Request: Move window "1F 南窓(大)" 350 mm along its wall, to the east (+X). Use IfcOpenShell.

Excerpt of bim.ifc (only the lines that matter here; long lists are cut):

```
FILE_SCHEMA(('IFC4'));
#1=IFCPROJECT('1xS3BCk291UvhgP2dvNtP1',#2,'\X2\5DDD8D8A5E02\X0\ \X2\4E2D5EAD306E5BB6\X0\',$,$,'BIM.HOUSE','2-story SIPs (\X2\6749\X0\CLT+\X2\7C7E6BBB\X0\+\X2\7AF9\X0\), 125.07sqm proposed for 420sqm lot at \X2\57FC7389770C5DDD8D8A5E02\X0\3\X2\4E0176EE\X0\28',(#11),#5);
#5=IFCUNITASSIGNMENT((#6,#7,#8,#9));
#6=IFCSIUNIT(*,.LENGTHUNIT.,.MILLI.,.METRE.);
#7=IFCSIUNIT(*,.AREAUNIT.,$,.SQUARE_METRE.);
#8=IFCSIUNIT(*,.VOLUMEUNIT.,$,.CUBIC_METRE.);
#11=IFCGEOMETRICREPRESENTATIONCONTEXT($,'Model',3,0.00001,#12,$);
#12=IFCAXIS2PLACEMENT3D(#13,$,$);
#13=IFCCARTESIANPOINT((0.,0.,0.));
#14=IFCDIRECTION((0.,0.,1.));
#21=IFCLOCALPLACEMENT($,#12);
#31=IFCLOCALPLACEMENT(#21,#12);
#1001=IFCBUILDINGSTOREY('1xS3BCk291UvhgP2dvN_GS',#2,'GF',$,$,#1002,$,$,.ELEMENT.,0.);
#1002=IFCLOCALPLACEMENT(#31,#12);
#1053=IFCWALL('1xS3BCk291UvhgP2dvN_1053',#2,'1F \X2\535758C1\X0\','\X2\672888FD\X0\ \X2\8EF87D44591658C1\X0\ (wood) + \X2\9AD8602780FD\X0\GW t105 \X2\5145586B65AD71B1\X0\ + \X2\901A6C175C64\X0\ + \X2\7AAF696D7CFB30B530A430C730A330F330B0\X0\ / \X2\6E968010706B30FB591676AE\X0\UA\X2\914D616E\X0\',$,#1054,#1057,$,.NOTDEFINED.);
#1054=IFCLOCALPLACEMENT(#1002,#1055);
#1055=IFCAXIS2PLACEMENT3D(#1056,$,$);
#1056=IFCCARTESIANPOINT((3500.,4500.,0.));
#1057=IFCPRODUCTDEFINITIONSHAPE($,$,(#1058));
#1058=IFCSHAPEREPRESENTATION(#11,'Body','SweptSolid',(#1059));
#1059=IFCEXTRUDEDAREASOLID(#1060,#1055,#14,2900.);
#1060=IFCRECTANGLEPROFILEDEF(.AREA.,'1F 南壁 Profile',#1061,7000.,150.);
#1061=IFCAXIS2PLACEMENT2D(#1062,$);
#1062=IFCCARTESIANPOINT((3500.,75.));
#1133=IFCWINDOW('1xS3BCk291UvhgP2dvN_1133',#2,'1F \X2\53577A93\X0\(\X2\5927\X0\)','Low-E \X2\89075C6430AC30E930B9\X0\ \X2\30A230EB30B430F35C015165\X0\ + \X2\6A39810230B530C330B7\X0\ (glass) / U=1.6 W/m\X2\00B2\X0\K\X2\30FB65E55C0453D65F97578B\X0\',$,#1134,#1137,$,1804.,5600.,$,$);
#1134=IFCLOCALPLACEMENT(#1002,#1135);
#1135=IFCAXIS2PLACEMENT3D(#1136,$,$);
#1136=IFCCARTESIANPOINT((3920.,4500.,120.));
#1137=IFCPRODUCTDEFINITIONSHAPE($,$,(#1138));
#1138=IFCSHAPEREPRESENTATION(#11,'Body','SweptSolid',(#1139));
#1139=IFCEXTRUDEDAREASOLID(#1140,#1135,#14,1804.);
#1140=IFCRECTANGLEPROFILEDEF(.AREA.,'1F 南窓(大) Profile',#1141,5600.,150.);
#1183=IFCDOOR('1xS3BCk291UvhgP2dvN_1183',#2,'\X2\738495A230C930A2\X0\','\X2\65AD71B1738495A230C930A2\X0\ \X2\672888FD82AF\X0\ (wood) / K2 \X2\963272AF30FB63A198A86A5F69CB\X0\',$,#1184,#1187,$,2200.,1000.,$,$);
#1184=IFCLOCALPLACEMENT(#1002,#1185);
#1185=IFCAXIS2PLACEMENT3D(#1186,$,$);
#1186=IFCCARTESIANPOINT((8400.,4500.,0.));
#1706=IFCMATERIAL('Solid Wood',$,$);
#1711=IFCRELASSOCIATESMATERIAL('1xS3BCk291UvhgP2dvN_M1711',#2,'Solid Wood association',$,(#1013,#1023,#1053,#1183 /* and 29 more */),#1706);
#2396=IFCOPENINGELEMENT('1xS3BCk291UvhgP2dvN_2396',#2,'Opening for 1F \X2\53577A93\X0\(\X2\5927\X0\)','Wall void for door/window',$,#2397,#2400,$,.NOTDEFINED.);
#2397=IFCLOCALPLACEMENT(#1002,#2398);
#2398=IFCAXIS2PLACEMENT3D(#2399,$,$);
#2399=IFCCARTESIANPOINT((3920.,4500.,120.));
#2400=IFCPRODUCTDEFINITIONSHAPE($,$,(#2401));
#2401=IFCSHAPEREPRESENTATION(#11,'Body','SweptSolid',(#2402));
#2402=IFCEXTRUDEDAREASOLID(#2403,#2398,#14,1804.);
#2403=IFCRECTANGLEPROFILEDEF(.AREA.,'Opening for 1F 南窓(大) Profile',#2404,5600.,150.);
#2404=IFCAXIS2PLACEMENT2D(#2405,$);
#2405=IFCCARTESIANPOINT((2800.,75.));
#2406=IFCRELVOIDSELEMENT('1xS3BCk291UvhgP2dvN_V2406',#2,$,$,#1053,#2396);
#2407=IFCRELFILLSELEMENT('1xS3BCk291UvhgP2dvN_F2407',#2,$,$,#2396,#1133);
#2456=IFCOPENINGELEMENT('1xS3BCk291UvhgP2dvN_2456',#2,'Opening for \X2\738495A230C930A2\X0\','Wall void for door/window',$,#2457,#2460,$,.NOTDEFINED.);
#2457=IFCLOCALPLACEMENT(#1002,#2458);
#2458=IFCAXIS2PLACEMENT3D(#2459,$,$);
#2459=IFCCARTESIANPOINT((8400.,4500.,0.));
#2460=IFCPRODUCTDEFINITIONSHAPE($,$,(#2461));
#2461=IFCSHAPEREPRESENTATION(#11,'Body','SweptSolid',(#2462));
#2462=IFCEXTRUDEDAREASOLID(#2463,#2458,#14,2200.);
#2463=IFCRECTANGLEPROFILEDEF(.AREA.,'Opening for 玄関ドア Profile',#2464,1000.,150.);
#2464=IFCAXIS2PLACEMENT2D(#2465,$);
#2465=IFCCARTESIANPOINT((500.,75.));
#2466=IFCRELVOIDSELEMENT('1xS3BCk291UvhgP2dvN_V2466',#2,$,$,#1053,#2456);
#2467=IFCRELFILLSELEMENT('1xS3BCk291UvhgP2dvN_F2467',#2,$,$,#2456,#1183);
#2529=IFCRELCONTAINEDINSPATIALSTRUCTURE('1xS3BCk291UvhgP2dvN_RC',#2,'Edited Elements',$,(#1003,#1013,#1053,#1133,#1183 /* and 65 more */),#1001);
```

```python
import ifcopenshell
import ifcopenshell.api.geometry
import ifcopenshell.util.placement

model = ifcopenshell.open("bim.ifc")

window = model.by_guid("1xS3BCk291UvhgP2dvN_1133")
opening = window.FillsVoids[0].RelatingOpeningElement
wall = opening.VoidsElements[0].RelatingBuildingElement

wall_matrix = ifcopenshell.util.placement.get_local_placement(wall.ObjectPlacement)
shift = wall_matrix[:3, 0] * 350.0
before = ifcopenshell.util.placement.get_local_placement(window.ObjectPlacement)[:3, 3].copy()

# The window is not placed relative to its opening, so move both.
for product in (opening, window):
    matrix = ifcopenshell.util.placement.get_local_placement(product.ObjectPlacement)
    matrix[:3, 3] += shift
    ifcopenshell.api.geometry.edit_object_placement(model, product=product, matrix=matrix, is_si=False)

after = ifcopenshell.util.placement.get_local_placement(window.ObjectPlacement)[:3, 3]
print("window moved by", (after - before).round(3) + 0.0)

model.write("bim_updated.ifc")
```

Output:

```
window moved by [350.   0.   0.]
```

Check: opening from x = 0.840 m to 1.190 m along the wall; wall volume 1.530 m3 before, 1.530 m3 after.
